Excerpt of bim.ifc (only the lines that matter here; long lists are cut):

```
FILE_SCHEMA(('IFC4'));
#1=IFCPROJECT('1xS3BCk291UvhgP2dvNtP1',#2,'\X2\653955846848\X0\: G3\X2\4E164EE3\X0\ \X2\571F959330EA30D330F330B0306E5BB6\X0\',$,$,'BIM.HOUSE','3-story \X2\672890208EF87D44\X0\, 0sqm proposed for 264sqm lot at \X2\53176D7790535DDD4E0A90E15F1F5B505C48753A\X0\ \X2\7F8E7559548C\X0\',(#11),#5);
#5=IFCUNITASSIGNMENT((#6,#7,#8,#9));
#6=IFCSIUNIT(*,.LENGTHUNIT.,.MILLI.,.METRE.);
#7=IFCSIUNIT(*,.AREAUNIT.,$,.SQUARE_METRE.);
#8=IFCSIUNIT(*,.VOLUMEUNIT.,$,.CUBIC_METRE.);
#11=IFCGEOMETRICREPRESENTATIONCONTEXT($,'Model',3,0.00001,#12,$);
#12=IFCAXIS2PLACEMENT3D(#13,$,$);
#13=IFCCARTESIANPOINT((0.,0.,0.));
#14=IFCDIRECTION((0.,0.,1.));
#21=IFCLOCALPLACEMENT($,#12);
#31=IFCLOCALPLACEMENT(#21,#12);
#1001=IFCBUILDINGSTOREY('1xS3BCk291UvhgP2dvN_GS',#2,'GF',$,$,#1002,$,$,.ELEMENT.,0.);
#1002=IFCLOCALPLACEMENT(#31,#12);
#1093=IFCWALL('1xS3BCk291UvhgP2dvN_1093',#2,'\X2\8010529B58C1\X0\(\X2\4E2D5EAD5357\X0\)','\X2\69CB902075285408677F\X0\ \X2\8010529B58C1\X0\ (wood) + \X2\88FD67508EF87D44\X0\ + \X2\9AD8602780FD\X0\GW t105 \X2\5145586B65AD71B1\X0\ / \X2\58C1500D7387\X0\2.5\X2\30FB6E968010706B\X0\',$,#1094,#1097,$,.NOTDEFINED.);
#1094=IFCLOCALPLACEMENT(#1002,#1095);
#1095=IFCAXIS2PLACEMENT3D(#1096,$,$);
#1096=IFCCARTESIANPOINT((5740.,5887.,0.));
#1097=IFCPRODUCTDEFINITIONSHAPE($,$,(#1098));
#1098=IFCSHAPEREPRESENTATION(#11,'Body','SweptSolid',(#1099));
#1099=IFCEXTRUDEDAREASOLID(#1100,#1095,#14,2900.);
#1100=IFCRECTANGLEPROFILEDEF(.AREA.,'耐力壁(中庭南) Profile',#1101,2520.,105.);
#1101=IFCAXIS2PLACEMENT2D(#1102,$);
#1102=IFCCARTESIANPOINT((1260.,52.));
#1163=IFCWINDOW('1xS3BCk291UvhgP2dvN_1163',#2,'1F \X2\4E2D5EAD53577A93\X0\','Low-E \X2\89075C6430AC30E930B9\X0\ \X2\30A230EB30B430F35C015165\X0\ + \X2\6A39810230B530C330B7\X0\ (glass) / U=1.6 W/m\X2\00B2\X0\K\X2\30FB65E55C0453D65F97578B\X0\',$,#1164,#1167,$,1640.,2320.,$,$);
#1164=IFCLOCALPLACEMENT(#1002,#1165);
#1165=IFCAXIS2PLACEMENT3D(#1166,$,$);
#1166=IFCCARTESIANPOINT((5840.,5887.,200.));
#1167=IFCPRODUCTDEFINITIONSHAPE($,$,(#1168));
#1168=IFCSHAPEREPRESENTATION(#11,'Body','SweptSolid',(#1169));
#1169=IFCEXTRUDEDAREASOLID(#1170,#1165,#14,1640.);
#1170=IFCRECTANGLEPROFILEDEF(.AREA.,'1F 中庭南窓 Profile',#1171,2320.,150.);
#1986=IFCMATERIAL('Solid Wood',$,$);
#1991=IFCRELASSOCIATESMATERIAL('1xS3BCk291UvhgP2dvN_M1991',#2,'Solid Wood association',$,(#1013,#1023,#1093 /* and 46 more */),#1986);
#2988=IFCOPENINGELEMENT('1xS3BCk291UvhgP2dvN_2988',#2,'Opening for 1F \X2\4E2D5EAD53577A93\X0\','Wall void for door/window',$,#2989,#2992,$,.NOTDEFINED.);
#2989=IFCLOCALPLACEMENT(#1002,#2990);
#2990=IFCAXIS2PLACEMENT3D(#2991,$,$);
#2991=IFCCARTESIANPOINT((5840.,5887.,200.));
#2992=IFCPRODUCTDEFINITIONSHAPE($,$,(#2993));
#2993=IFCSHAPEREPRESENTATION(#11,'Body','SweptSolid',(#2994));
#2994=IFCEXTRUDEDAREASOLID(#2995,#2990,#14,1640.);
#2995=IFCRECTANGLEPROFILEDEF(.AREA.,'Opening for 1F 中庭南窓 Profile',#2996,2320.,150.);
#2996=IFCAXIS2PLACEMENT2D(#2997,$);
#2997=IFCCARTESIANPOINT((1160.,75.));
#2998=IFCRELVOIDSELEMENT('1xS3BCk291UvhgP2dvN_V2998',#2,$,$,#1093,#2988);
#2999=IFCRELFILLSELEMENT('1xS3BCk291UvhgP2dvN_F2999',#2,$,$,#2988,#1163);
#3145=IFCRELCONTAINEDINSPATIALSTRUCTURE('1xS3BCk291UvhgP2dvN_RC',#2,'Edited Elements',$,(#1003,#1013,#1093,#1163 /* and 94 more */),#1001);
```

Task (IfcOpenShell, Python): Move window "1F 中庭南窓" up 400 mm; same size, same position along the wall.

```python
import numpy as np
import ifcopenshell
import ifcopenshell.api.geometry
import ifcopenshell.util.placement
import ifcopenshell.util.unit

model = ifcopenshell.open("bim.ifc")
unit_scale = ifcopenshell.util.unit.calculate_unit_scale(model)

window = model.by_guid("1xS3BCk291UvhgP2dvN_1163")
opening = window.FillsVoids[0].RelatingOpeningElement
dz = 400.0

shift = np.array([0.0, 0.0, dz])
# The window is not placed relative to its opening, so move both.
for product in (opening, window):
    matrix = ifcopenshell.util.placement.get_local_placement(product.ObjectPlacement)
    matrix[:3, 3] += shift
    ifcopenshell.api.geometry.edit_object_placement(model, product=product, matrix=matrix, is_si=False)

print(f"moved by {dz * unit_scale:+.3f} m")

model.write("bim-out.ifc")
```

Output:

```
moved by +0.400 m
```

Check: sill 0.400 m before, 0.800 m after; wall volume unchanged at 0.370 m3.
